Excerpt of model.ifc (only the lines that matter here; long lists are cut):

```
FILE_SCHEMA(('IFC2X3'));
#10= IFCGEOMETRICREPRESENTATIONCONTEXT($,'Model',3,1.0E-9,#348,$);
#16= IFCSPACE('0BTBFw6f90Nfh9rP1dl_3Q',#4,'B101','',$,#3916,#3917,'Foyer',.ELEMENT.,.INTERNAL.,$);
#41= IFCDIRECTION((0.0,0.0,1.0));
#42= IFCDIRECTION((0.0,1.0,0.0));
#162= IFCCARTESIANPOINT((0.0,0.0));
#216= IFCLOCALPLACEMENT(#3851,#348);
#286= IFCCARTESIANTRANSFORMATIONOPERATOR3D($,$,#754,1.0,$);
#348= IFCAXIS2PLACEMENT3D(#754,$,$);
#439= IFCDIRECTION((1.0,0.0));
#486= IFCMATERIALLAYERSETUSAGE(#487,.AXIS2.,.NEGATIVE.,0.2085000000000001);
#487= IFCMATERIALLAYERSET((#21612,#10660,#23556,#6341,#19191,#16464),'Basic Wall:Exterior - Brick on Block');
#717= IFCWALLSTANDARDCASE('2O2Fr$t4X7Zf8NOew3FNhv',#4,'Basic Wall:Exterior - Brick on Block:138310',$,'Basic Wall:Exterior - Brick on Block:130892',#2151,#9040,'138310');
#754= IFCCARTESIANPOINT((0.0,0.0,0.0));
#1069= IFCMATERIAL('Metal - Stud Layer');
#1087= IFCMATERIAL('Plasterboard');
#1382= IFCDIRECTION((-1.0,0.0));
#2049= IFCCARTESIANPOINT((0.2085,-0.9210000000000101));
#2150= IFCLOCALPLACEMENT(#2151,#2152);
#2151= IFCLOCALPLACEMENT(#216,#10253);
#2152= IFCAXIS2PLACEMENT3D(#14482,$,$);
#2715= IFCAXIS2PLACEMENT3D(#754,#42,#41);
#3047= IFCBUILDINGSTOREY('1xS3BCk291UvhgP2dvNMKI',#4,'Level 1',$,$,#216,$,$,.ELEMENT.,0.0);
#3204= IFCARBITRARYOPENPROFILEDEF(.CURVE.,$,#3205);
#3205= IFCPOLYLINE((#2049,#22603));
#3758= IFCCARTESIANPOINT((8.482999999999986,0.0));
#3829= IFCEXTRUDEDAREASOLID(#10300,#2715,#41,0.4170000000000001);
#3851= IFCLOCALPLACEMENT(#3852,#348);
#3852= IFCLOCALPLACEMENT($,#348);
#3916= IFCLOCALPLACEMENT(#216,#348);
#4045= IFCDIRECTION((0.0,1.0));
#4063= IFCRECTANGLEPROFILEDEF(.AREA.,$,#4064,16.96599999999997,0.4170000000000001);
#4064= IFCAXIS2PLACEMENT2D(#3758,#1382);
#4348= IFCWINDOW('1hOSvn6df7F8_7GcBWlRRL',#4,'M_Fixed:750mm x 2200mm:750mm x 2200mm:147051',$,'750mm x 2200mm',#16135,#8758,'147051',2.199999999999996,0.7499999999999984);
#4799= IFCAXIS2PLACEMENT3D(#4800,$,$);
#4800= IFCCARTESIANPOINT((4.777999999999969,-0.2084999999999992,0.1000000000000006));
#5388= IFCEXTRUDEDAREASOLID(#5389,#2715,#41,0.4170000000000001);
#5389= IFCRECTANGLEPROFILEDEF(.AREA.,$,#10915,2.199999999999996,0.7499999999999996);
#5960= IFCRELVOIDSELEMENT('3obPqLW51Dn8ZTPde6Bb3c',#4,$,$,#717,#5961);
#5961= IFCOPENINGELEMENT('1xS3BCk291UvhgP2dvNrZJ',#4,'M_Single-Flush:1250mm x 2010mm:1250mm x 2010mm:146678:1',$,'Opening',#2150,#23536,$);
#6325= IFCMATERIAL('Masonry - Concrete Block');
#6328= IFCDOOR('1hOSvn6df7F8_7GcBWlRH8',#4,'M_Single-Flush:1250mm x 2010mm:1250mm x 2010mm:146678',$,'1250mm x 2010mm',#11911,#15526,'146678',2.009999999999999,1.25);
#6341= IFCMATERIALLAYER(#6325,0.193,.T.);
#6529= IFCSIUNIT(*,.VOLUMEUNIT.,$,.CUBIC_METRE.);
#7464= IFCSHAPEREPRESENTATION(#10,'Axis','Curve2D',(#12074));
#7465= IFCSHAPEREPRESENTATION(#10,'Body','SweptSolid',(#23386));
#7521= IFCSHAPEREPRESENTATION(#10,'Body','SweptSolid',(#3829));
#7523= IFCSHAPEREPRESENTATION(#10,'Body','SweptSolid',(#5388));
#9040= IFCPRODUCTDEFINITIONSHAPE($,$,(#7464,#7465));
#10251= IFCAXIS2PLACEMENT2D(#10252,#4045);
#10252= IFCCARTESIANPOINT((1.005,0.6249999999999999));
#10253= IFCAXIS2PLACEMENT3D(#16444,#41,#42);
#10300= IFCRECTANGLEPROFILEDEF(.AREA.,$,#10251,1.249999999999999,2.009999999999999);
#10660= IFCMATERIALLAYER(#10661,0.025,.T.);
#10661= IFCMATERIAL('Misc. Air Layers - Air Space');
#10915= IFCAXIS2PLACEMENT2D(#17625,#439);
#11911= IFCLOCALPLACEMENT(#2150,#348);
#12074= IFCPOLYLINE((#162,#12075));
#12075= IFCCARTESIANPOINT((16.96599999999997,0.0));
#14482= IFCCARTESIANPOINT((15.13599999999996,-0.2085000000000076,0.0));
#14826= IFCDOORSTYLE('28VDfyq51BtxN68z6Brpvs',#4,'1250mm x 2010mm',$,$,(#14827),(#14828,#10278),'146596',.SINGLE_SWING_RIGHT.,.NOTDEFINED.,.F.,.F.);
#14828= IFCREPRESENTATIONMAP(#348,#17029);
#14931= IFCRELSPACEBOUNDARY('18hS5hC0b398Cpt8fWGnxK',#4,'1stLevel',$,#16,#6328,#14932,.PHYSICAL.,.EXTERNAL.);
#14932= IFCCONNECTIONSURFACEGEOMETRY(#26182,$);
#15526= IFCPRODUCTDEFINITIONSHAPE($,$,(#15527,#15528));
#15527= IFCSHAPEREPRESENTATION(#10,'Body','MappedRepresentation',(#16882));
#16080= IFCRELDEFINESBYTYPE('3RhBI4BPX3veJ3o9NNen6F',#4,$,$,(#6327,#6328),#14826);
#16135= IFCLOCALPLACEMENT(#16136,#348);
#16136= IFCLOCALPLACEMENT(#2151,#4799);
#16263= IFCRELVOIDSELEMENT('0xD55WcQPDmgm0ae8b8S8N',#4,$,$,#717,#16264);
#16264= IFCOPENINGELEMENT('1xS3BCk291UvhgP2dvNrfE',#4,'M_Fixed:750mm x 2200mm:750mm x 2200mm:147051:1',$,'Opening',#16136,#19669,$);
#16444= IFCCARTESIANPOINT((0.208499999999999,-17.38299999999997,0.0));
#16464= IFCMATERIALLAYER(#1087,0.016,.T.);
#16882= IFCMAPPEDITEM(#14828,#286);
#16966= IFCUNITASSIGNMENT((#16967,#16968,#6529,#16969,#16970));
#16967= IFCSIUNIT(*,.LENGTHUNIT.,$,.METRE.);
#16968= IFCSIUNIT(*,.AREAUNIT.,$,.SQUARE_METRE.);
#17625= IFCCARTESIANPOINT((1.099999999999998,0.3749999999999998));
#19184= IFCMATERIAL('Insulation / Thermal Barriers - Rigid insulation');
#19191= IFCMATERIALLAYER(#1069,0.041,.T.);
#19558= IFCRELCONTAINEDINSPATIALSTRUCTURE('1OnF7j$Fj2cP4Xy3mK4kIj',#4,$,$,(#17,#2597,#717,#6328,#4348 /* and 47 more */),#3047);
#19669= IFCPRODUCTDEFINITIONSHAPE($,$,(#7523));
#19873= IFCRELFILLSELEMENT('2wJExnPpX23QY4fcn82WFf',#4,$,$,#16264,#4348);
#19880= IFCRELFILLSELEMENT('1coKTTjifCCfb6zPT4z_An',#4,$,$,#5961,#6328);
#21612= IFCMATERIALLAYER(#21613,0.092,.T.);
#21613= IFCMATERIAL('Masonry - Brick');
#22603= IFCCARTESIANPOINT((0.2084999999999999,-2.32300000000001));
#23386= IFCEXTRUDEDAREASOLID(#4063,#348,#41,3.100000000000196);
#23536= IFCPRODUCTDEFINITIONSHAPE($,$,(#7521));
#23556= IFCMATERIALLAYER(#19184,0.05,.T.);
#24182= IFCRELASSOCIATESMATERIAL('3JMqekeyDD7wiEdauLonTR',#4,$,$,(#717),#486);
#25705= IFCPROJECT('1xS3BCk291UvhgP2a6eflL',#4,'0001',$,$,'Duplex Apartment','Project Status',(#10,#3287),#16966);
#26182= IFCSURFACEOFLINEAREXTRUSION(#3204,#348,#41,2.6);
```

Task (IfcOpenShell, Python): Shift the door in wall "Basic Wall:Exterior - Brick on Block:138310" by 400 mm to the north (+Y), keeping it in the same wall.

```python
import numpy as np
import ifcopenshell
import ifcopenshell.api.geometry
import ifcopenshell.util.placement

model = ifcopenshell.open("model.ifc")

door = model.by_guid("1hOSvn6df7F8_7GcBWlRH8")
opening = door.FillsVoids[0].RelatingOpeningElement
wall = opening.VoidsElements[0].RelatingBuildingElement

wall_matrix = ifcopenshell.util.placement.get_local_placement(wall.ObjectPlacement)
shift = wall_matrix[:3, 0] * 0.4
before = ifcopenshell.util.placement.get_local_placement(door.ObjectPlacement)[:3, 3].copy()

# The door is placed relative to its opening, so it follows when the opening moves.
matrix = ifcopenshell.util.placement.get_local_placement(opening.ObjectPlacement)
matrix[:3, 3] += shift
ifcopenshell.api.geometry.edit_object_placement(
    model, product=opening, matrix=matrix, is_si=False, should_transform_children=True
)

# Space boundary surfaces are stored in each space's coordinates; move them too.
for rel in door.ProvidesBoundaries:
    if not rel.ConnectionGeometry:
        continue
    surface = rel.ConnectionGeometry.SurfaceOnRelatingElement
    space_matrix = ifcopenshell.util.placement.get_local_placement(rel.RelatingSpace.ObjectPlacement)
    point = np.array(surface.Position.Location.Coordinates) + space_matrix[:3, :3].T @ shift
    surface.Position = model.createIfcAxis2Placement3D(
        model.createIfcCartesianPoint(point.tolist()), surface.Position.Axis, surface.Position.RefDirection
    )

after = ifcopenshell.util.placement.get_local_placement(door.ObjectPlacement)[:3, 3]
print("door moved by", (after - before).round(3) + 0.0)

model.write("model_edited.ifc")
```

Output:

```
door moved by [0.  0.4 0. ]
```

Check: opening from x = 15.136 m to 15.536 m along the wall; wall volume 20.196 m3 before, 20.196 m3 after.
